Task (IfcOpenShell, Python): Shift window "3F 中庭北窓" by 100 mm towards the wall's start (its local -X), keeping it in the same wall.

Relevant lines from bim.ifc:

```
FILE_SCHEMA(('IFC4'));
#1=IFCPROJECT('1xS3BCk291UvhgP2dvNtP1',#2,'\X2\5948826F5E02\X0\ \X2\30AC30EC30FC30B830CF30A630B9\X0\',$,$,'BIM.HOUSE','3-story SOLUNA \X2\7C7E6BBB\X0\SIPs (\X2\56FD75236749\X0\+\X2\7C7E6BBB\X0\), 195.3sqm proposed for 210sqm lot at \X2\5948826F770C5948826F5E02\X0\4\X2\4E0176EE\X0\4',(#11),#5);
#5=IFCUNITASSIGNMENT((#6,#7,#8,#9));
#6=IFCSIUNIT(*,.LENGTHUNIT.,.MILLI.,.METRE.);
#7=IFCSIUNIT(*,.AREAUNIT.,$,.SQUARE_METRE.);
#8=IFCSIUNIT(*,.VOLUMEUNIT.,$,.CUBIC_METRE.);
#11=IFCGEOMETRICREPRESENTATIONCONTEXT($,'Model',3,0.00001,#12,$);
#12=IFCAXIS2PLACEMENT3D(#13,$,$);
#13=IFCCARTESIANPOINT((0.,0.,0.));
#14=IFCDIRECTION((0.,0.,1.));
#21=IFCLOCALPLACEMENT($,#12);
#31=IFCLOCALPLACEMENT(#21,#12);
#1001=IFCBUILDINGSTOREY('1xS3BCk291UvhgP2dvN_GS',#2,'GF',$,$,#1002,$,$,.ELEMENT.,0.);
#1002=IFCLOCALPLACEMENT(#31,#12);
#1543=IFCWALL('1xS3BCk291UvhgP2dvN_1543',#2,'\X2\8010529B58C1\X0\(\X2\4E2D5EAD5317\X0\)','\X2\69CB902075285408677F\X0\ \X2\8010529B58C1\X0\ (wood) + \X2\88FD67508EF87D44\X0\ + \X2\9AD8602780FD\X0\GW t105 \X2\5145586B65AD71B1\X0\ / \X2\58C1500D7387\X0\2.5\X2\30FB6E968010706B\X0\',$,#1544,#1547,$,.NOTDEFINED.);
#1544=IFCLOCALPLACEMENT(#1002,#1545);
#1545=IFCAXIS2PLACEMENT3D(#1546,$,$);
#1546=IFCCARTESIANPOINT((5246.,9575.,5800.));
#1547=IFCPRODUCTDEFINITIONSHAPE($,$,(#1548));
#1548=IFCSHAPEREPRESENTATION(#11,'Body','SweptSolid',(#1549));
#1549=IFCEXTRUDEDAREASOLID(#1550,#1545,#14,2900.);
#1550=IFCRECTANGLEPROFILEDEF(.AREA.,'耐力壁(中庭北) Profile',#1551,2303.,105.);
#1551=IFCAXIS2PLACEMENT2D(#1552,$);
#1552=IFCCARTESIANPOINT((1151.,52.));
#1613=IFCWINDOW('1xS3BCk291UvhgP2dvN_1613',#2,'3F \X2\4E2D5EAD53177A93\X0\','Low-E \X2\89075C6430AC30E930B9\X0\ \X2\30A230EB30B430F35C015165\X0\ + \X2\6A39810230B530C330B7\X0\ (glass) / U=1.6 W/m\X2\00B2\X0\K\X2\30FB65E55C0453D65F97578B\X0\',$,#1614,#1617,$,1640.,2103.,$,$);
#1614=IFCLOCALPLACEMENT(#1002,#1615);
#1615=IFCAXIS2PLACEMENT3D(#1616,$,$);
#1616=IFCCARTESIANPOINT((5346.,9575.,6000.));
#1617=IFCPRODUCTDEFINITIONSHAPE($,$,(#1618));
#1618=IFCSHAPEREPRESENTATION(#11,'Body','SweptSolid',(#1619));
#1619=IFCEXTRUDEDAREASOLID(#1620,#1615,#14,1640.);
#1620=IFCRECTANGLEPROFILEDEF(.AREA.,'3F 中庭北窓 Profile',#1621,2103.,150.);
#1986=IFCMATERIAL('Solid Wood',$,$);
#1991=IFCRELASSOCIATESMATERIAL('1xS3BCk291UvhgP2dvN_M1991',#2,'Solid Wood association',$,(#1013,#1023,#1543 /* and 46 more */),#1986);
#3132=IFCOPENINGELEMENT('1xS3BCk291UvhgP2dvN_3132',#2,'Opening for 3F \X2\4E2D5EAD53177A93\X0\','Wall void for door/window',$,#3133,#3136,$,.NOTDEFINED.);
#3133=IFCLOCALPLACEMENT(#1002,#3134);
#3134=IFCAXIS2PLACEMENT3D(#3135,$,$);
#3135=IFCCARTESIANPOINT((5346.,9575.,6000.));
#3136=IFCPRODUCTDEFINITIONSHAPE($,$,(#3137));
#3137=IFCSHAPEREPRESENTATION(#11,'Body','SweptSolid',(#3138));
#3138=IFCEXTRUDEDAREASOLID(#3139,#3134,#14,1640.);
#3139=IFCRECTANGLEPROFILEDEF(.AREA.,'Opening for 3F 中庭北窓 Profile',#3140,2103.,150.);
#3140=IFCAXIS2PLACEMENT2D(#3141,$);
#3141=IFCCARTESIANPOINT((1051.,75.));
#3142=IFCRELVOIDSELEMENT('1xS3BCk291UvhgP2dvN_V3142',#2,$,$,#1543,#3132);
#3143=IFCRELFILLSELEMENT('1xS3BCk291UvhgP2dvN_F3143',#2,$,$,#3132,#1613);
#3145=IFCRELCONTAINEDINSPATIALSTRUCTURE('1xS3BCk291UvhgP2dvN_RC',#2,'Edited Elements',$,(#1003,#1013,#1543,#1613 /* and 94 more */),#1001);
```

```python
import ifcopenshell
import ifcopenshell.api.geometry
import ifcopenshell.util.placement
import ifcopenshell.util.unit

model = ifcopenshell.open("bim.ifc")
unit_scale = ifcopenshell.util.unit.calculate_unit_scale(model)

window = model.by_guid("1xS3BCk291UvhgP2dvN_1613")
opening = window.FillsVoids[0].RelatingOpeningElement
wall = opening.VoidsElements[0].RelatingBuildingElement

wall_matrix = ifcopenshell.util.placement.get_local_placement(wall.ObjectPlacement)
shift = wall_matrix[:3, 0] * -0.1 / unit_scale
before = ifcopenshell.util.placement.get_local_placement(window.ObjectPlacement)[:3, 3].copy()

# The window is not placed relative to its opening, so move both.
for product in (opening, window):
    matrix = ifcopenshell.util.placement.get_local_placement(product.ObjectPlacement)
    matrix[:3, 3] += shift
    ifcopenshell.api.geometry.edit_object_placement(model, product=product, matrix=matrix, is_si=False)

after = ifcopenshell.util.placement.get_local_placement(window.ObjectPlacement)[:3, 3]
print("window moved by", (after - before).round(3) + 0.0)

model.write("bim_rev.ifc")
```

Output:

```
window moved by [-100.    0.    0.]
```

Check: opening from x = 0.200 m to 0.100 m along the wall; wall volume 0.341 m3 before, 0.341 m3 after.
